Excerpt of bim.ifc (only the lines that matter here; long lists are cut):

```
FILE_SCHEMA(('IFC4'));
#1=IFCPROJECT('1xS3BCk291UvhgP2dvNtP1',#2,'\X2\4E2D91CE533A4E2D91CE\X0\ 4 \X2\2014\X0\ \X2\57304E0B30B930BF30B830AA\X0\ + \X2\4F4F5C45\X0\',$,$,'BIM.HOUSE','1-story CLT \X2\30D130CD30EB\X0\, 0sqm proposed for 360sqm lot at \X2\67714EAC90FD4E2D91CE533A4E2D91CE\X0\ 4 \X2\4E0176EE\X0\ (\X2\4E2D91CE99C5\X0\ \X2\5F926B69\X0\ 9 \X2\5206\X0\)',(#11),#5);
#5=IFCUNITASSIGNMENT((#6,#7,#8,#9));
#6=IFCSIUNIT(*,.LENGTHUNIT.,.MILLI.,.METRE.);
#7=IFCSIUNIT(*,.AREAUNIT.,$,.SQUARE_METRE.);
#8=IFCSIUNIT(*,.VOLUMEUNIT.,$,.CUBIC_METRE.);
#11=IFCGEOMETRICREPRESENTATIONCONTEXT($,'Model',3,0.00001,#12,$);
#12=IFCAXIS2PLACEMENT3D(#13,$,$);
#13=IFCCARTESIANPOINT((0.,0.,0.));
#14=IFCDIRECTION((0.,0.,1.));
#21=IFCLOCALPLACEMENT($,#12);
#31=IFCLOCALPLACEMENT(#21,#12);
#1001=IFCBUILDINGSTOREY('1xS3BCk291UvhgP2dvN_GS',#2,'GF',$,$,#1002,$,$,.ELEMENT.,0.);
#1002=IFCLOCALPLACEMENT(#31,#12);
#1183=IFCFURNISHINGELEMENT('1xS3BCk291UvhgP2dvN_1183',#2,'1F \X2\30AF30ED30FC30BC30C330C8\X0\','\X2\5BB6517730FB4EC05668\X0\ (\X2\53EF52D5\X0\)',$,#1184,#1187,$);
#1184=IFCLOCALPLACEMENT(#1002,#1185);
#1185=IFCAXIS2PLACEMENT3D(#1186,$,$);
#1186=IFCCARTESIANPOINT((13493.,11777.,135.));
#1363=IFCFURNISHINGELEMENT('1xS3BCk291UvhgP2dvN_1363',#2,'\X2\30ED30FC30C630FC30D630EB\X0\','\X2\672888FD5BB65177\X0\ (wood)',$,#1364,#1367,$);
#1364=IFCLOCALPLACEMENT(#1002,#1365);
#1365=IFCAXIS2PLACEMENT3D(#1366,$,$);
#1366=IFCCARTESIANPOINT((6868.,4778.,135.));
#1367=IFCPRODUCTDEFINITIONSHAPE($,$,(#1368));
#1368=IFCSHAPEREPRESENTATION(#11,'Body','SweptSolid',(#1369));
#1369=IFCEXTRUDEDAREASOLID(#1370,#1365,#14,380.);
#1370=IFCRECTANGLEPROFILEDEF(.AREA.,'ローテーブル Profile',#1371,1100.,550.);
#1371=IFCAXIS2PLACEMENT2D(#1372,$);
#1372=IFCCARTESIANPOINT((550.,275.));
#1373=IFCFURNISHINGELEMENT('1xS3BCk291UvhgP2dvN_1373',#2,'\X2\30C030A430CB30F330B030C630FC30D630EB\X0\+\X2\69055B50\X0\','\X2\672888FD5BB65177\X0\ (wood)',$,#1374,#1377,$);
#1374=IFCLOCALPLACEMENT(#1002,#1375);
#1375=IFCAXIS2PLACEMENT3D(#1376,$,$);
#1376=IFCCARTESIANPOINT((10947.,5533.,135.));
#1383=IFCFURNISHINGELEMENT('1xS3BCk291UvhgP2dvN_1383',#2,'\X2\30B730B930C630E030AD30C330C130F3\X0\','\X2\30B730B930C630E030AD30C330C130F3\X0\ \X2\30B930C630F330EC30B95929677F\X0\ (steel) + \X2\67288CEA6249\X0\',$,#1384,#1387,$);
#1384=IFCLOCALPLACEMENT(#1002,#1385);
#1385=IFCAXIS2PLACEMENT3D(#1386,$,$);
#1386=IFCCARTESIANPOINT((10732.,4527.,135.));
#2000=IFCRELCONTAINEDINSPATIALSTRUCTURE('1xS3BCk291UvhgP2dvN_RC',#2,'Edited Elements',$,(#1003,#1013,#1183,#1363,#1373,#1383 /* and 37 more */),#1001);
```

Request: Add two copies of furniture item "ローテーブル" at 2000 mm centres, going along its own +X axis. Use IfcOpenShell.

```python
import ifcopenshell
import ifcopenshell.api.geometry
import ifcopenshell.api.root
import ifcopenshell.util.element
import ifcopenshell.util.placement
import ifcopenshell.util.unit

model = ifcopenshell.open("bim.ifc")
unit_scale = ifcopenshell.util.unit.calculate_unit_scale(model)


def reuse_history(source, copy):
    """copy_class also copies each property set's owner history, people and application; keep the originals."""
    for rel in copy.IsDefinedBy:
        if rel.is_a("IfcRelDefinesByProperties") and (history := rel.RelatingPropertyDefinition.OwnerHistory):
            rel.RelatingPropertyDefinition.OwnerHistory = source.OwnerHistory
            ifcopenshell.util.element.remove_deep2(model, history)


source = model.by_id(1363)
base = ifcopenshell.util.placement.get_local_placement(source.ObjectPlacement)
step = base[:3, 0] * 2 / unit_scale

for i in range(1, 3):
    copy = ifcopenshell.api.root.copy_class(model, product=source)
    copy.Representation = ifcopenshell.util.element.copy_deep(
        model, source.Representation, exclude=["IfcGeometricRepresentationContext", "IfcRepresentationMap"]
    )
    reuse_history(source, copy)
    matrix = base.copy()
    matrix[:3, 3] += i * step
    print("added at", matrix[:3, 3].round(3) + 0.0)
    ifcopenshell.api.geometry.edit_object_placement(model, product=copy, matrix=matrix, is_si=False)

model.write("bim_edited.ifc")
```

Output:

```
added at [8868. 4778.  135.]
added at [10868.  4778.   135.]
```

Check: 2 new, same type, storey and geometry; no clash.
